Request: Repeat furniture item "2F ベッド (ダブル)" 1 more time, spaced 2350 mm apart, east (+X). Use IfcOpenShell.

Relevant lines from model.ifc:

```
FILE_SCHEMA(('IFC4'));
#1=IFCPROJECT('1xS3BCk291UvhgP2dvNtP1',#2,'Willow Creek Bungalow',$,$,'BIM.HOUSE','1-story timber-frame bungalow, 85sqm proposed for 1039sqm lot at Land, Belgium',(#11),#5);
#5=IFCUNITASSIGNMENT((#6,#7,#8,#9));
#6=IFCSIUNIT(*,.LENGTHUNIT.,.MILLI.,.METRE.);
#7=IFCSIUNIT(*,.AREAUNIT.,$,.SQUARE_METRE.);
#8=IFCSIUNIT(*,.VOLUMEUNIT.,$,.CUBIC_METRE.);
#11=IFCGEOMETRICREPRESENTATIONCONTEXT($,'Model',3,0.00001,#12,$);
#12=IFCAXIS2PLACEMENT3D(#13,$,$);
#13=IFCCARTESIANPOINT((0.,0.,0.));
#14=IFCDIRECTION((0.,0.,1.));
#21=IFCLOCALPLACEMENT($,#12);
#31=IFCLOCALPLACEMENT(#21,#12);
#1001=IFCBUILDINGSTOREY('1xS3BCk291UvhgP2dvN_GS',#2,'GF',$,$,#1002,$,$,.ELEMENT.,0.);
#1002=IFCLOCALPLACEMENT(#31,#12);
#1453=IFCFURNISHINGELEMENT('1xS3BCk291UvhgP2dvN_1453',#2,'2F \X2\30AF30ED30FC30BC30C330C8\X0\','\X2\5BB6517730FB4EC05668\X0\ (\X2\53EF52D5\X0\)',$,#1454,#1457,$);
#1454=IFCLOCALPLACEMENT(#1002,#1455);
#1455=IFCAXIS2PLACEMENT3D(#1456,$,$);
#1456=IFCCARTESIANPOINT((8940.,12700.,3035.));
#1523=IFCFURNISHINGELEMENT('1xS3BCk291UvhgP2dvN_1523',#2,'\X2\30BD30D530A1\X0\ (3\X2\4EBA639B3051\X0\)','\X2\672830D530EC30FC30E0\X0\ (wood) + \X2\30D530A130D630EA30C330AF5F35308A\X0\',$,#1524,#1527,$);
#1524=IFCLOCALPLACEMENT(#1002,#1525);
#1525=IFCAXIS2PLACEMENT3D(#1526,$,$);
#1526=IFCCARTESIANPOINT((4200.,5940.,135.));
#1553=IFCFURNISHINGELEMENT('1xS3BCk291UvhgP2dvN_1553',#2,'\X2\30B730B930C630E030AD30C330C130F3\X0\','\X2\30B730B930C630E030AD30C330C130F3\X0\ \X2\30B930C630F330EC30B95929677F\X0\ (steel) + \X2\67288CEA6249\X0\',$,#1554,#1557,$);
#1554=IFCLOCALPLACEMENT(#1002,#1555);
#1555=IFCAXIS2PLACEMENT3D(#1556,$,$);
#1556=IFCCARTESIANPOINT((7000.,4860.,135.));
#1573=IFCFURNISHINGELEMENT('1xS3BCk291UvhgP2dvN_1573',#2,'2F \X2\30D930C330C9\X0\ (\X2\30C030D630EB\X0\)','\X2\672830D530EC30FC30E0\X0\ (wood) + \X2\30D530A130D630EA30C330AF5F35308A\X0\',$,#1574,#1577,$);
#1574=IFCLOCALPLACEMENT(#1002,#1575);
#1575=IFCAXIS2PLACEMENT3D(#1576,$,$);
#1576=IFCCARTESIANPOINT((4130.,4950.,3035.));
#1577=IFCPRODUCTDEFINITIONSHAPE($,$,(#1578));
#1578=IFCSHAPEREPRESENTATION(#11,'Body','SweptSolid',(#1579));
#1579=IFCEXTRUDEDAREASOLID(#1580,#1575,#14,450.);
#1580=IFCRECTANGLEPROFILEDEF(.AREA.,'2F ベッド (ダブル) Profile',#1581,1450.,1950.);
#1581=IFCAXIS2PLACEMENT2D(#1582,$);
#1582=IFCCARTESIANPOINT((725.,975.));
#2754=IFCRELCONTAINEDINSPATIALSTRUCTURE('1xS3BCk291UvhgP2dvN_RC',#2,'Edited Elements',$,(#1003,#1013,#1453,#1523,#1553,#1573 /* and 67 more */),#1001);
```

```python
import numpy as np
import ifcopenshell
import ifcopenshell.api.geometry
import ifcopenshell.api.root
import ifcopenshell.util.element
import ifcopenshell.util.placement
import ifcopenshell.util.unit

model = ifcopenshell.open("model.ifc")
unit_scale = ifcopenshell.util.unit.calculate_unit_scale(model)


def reuse_history(source, copy):
    """copy_class also copies each property set's owner history, people and application; keep the originals."""
    for rel in copy.IsDefinedBy:
        if rel.is_a("IfcRelDefinesByProperties") and (history := rel.RelatingPropertyDefinition.OwnerHistory):
            rel.RelatingPropertyDefinition.OwnerHistory = source.OwnerHistory
            ifcopenshell.util.element.remove_deep2(model, history)


source = model.by_guid("1xS3BCk291UvhgP2dvN_1573")
base = ifcopenshell.util.placement.get_local_placement(source.ObjectPlacement)
step = np.array([1.0, 0.0, 0.0]) * 2.35 / unit_scale

for i in range(1, 2):
    copy = ifcopenshell.api.root.copy_class(model, product=source)
    copy.Representation = ifcopenshell.util.element.copy_deep(
        model, source.Representation, exclude=["IfcGeometricRepresentationContext", "IfcRepresentationMap"]
    )
    reuse_history(source, copy)
    matrix = base.copy()
    matrix[:3, 3] += i * step
    print("added at", matrix[:3, 3].round(3) + 0.0)
    ifcopenshell.api.geometry.edit_object_placement(model, product=copy, matrix=matrix, is_si=False)

model.write("model_v2.ifc")
```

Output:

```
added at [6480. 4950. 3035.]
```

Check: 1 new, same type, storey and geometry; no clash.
